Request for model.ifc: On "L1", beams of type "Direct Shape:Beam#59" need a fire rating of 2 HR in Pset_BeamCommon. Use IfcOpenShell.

First a look at what the model holds.

```python
import ifcopenshell
import ifcopenshell.util.element

model = ifcopenshell.open("model.ifc")
print(model.schema)
storey = next(s for s in model.by_type("IfcBuildingStorey") if s.Name == "L1")
beams = [e for e in ifcopenshell.util.element.get_decomposition(storey) if e.is_a("IfcBeam")]
seen = {}
for e in beams:
    element_type = ifcopenshell.util.element.get_type(e)
    key = (element_type.Name if element_type != e and element_type else None, ifcopenshell.util.element.get_pset(e, "Pset_BeamCommon", "FireRating"))
    seen[key] = seen.get(key, 0) + 1
for (name, value), count in sorted(seen.items(), key=str):
    print(count, "x", name, "|", value)
```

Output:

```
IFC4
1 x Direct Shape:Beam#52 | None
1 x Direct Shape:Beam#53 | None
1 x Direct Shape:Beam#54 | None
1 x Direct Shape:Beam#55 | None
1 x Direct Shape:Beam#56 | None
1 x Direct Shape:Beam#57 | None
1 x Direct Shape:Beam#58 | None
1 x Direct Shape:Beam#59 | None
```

```python
import ifcopenshell
import ifcopenshell.api.pset
import ifcopenshell.util.element

model = ifcopenshell.open("model.ifc")

storey = next(s for s in model.by_type("IfcBuildingStorey") if s.Name == "L1")
beams = [e for e in ifcopenshell.util.element.get_decomposition(storey) if e.is_a("IfcBeam")]

count = 0
for e in beams:
    element_type = ifcopenshell.util.element.get_type(e)
    if element_type in (None, e) or element_type.Name != "Direct Shape:Beam#59":
        continue
    # add_pset returns the element's existing set when there is one.
    pset = ifcopenshell.api.pset.add_pset(model, product=e, name="Pset_BeamCommon")
    ifcopenshell.api.pset.edit_pset(model, pset=pset, properties={"FireRating": "2 HR"})
    count += 1

print(count, "beams updated")

model.write("model_edited.ifc")
```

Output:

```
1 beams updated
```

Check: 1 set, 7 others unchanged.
